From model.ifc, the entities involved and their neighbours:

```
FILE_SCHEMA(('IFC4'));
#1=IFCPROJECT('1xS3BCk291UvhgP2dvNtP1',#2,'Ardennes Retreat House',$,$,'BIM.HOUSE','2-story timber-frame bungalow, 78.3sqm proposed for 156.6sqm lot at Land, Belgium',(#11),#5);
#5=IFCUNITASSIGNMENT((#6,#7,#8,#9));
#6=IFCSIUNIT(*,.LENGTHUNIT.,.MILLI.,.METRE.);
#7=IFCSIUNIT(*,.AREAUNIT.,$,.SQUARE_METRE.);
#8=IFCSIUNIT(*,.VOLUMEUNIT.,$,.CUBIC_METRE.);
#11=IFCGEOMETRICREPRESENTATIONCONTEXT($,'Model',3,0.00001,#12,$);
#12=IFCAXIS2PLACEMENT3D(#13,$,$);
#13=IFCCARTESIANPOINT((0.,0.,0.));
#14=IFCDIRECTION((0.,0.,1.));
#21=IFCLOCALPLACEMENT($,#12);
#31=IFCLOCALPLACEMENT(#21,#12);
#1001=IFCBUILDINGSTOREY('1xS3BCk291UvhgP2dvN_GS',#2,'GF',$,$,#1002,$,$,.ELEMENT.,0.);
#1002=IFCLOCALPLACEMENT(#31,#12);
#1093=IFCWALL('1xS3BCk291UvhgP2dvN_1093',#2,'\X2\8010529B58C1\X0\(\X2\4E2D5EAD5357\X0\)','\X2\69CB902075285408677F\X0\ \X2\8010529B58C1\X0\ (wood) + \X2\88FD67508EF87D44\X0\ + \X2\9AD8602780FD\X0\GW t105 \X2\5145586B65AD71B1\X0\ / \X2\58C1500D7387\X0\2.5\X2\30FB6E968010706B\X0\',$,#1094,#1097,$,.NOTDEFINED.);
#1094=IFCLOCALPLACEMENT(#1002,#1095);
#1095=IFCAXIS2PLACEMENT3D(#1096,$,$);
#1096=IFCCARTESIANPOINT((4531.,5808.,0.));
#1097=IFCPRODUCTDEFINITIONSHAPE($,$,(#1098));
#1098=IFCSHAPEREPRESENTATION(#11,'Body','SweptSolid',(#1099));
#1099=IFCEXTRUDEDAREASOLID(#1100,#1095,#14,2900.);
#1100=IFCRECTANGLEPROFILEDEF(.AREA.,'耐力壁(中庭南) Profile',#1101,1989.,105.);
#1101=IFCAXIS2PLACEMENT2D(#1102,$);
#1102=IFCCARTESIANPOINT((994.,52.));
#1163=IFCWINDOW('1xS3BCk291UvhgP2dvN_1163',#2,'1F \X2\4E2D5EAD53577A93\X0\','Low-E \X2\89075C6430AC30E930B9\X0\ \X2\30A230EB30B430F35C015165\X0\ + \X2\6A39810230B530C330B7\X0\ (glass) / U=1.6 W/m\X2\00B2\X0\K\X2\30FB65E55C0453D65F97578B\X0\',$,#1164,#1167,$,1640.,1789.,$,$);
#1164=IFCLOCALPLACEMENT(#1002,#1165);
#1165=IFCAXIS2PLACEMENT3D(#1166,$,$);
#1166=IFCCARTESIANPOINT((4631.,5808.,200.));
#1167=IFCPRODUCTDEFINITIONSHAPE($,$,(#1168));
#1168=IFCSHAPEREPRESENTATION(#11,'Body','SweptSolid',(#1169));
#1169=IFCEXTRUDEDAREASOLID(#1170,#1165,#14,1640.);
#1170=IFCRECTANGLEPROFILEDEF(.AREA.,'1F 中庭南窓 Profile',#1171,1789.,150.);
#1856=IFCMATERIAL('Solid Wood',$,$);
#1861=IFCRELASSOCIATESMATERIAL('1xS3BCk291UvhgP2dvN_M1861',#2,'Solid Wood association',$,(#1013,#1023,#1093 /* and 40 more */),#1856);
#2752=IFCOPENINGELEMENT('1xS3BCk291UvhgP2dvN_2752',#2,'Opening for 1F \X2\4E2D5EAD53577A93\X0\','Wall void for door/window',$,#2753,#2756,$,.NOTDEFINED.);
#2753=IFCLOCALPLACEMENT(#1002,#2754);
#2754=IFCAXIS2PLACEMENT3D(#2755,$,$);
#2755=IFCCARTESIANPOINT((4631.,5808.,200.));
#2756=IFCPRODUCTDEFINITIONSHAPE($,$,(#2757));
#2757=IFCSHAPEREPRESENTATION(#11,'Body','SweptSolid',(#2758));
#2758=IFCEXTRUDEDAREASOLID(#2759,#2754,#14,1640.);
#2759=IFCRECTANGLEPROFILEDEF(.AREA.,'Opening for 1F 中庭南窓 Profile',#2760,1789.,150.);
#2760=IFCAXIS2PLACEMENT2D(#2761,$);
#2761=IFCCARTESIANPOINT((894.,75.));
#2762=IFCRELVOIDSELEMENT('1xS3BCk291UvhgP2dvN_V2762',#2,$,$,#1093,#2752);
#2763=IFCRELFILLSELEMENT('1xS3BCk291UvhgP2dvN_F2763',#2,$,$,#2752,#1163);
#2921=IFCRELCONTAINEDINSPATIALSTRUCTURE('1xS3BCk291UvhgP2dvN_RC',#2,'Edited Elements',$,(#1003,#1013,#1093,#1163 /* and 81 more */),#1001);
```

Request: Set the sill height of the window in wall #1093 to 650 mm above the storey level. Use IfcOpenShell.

```python
import numpy as np
import ifcopenshell
import ifcopenshell.api.geometry
import ifcopenshell.geom
import ifcopenshell.util.element
import ifcopenshell.util.placement
import ifcopenshell.util.shape
import ifcopenshell.util.unit

model = ifcopenshell.open("model.ifc")
unit_scale = ifcopenshell.util.unit.calculate_unit_scale(model)

window = model.by_guid("1xS3BCk291UvhgP2dvN_1163")
opening = window.FillsVoids[0].RelatingOpeningElement
storey = ifcopenshell.util.element.get_container(window, ifc_class="IfcBuildingStorey")
level = ifcopenshell.util.placement.get_local_placement(storey.ObjectPlacement)[2, 3]

# The opening's origin need not be at the sill, so measure its lowest point.
shape = ifcopenshell.geom.create_shape(ifcopenshell.geom.settings(), opening)
bottom = ifcopenshell.util.shape.get_shape_bottom_elevation(shape, shape.geometry) / unit_scale
dz = level + 0.65 / unit_scale - bottom

shift = np.array([0.0, 0.0, dz])
# The window is not placed relative to its opening, so move both.
for product in (opening, window):
    matrix = ifcopenshell.util.placement.get_local_placement(product.ObjectPlacement)
    matrix[:3, 3] += shift
    ifcopenshell.api.geometry.edit_object_placement(model, product=product, matrix=matrix, is_si=False)

print(f"moved by {dz * unit_scale:+.3f} m")

model.write("model-out.ifc")
```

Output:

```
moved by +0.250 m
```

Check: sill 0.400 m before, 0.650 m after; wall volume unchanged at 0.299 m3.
